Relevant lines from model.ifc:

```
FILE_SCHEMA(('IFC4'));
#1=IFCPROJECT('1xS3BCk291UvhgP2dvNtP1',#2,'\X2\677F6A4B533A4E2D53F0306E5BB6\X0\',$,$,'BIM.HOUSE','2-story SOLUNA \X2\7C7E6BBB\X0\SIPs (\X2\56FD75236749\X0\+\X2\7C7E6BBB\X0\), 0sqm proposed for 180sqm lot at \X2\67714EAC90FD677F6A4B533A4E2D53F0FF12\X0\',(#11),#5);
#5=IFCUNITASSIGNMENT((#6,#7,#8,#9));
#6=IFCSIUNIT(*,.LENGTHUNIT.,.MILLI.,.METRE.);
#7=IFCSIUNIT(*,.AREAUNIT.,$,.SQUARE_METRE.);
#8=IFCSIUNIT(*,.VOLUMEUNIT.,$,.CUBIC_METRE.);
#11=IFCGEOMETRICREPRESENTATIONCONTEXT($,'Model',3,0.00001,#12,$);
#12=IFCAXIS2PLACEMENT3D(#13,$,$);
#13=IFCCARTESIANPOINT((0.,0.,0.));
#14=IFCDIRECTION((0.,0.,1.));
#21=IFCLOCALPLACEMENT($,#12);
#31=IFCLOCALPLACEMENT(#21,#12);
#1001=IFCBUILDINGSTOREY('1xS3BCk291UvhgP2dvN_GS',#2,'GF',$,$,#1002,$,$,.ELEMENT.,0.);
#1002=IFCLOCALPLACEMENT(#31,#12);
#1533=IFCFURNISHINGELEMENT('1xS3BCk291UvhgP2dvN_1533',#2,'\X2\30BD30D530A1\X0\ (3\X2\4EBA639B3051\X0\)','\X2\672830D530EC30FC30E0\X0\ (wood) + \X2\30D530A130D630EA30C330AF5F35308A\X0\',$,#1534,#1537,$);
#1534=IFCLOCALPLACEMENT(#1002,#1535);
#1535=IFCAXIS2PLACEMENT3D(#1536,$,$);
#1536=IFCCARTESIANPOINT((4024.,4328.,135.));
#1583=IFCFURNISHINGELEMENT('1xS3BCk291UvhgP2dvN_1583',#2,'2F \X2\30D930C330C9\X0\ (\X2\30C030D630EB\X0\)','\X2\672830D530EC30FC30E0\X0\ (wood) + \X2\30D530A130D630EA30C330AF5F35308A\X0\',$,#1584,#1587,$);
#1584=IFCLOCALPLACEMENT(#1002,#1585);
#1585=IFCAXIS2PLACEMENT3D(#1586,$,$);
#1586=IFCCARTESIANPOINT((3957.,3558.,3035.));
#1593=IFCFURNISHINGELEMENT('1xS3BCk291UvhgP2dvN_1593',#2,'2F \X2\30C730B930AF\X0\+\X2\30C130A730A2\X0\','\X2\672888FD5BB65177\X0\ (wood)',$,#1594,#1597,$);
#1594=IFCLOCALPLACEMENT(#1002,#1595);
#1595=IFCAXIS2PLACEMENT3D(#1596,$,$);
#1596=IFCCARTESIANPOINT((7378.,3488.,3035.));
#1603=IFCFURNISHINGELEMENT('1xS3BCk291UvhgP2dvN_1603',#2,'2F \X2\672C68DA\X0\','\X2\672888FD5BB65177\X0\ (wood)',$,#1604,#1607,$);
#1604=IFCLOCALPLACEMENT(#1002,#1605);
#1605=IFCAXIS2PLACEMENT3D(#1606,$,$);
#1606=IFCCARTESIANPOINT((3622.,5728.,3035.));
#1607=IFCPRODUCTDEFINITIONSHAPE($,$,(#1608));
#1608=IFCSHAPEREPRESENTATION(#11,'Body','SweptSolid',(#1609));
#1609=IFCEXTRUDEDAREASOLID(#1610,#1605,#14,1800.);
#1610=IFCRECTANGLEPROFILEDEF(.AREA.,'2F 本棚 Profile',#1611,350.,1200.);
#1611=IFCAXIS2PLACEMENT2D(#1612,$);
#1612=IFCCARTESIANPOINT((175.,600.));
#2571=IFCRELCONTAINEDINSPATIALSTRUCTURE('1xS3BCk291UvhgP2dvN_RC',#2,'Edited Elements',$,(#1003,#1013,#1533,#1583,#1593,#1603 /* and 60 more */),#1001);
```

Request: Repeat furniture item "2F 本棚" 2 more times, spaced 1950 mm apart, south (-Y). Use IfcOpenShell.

```python
import numpy as np
import ifcopenshell
import ifcopenshell.api.geometry
import ifcopenshell.api.root
import ifcopenshell.util.element
import ifcopenshell.util.placement
import ifcopenshell.util.unit

model = ifcopenshell.open("model.ifc")
unit_scale = ifcopenshell.util.unit.calculate_unit_scale(model)


def reuse_history(source, copy):
    """copy_class also copies each property set's owner history, people and application; keep the originals."""
    for rel in copy.IsDefinedBy:
        if rel.is_a("IfcRelDefinesByProperties") and (history := rel.RelatingPropertyDefinition.OwnerHistory):
            rel.RelatingPropertyDefinition.OwnerHistory = source.OwnerHistory
            ifcopenshell.util.element.remove_deep2(model, history)


source = model.by_id(1603)
base = ifcopenshell.util.placement.get_local_placement(source.ObjectPlacement)
step = np.array([0.0, -1.0, 0.0]) * 1.95 / unit_scale

for i in range(1, 3):
    copy = ifcopenshell.api.root.copy_class(model, product=source)
    copy.Representation = ifcopenshell.util.element.copy_deep(
        model, source.Representation, exclude=["IfcGeometricRepresentationContext", "IfcRepresentationMap"]
    )
    reuse_history(source, copy)
    matrix = base.copy()
    matrix[:3, 3] += i * step
    print("added at", matrix[:3, 3].round(3) + 0.0)
    ifcopenshell.api.geometry.edit_object_placement(model, product=copy, matrix=matrix, is_si=False)

model.write("model-out.ifc")
```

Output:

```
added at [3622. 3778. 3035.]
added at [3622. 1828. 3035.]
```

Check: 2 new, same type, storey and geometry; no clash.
